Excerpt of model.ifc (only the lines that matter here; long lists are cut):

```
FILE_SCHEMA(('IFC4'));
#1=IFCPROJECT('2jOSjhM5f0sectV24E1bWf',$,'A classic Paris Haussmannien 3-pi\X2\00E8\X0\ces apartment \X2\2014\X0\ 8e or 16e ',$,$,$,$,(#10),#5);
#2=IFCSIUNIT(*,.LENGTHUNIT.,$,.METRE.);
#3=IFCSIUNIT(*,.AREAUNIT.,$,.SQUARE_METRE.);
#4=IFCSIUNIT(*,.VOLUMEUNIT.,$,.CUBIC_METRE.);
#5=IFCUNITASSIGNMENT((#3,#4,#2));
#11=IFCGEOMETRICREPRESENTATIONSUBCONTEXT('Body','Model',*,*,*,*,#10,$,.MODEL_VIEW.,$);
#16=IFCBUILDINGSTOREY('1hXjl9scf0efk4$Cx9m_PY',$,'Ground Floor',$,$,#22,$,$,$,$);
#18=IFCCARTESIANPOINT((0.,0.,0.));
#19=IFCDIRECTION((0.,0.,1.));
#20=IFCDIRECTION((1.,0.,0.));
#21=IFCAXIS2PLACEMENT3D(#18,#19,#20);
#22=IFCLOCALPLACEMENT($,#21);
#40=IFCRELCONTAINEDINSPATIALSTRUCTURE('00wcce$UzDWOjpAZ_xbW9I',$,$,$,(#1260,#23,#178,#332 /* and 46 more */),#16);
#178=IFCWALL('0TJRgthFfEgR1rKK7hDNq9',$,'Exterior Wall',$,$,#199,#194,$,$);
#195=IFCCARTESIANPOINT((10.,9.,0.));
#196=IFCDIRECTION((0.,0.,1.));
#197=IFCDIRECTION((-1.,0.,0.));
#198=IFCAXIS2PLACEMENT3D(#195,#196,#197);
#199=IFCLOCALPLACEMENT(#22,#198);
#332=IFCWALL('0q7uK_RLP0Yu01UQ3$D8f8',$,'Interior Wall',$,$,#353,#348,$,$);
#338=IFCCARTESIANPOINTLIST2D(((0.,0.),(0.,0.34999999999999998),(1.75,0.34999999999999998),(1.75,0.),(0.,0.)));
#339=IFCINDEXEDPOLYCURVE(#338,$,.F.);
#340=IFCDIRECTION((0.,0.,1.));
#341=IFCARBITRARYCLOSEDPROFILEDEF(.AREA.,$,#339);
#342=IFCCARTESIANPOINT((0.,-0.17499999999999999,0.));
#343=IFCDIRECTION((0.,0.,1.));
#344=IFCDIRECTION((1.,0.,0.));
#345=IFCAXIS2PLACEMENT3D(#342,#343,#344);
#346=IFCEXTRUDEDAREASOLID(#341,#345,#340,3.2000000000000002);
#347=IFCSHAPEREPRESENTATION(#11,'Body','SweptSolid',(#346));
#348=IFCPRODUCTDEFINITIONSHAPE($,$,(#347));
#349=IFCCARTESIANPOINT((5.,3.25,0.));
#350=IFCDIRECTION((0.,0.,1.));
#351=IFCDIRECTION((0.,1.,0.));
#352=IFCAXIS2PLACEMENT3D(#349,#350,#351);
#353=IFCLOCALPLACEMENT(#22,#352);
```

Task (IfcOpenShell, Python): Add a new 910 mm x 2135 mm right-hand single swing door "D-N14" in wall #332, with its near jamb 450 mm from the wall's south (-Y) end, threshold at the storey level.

```python
import numpy as np
import ifcopenshell
import ifcopenshell.api.feature
import ifcopenshell.api.geometry
import ifcopenshell.api.root
import ifcopenshell.api.spatial
import ifcopenshell.geom
import ifcopenshell.util.element
import ifcopenshell.util.placement
import ifcopenshell.util.representation
import ifcopenshell.util.shape
import ifcopenshell.util.unit

model = ifcopenshell.open("model.ifc")
unit_scale = ifcopenshell.util.unit.calculate_unit_scale(model)
settings = ifcopenshell.geom.settings()


def volume(element):
    """Net volume in cubic metres, openings subtracted."""
    shape = ifcopenshell.geom.create_shape(settings, element)
    return ifcopenshell.util.shape.get_volume(shape.geometry)


wall = model.by_guid("0q7uK_RLP0Yu01UQ3$D8f8")
storey = ifcopenshell.util.element.get_container(wall, ifc_class="IfcBuildingStorey")
context = ifcopenshell.util.representation.get_context(model, "Model", "Body", "MODEL_VIEW")
before = volume(wall)

width, height, from_end, sill = 0.91, 2.135, 0.45, 0.0  # metres

# The wall runs along its own X axis, and the end named is its -X end.
wall_shape = ifcopenshell.geom.create_shape(settings, wall)
x, y, z = ifcopenshell.util.shape.get_vertices(wall_shape.geometry).T
start = x.min() + from_end
face, thickness = float(y.min()), float(y.max() - y.min())
wall_matrix = ifcopenshell.util.placement.get_local_placement(wall.ObjectPlacement)
level = ifcopenshell.util.placement.get_local_placement(storey.ObjectPlacement)[2, 3]


def in_wall(x, y):
    """Placement at x, y metres in the wall's axes, at sill height."""
    matrix = wall_matrix.copy()
    matrix[:, 3] = wall_matrix @ np.array([x / unit_scale, y / unit_scale, 0.0, 1.0])
    matrix[2, 3] = level + sill / unit_scale
    return matrix


# Opening: a box that overshoots both wall faces by 50 mm.
opening = ifcopenshell.api.root.create_entity(model, ifc_class="IfcOpeningElement", predefined_type="OPENING")
box = ifcopenshell.api.geometry.add_wall_representation(
    model, context=context, length=width, height=height, thickness=thickness + 0.1
)
ifcopenshell.api.geometry.assign_representation(model, product=opening, representation=box)
ifcopenshell.api.geometry.edit_object_placement(model, product=opening, matrix=in_wall(start, face - 0.05), is_si=False)
ifcopenshell.api.feature.add_feature(model, feature=opening, element=wall)

door = ifcopenshell.api.root.create_entity(model, ifc_class="IfcDoor", name="D-N14", predefined_type="DOOR")
door.OverallWidth, door.OverallHeight = width / unit_scale, height / unit_scale
door.OperationType = "SINGLE_SWING_RIGHT"
body = ifcopenshell.api.geometry.add_door_representation(
    model,
    context=context,
    overall_width=door.OverallWidth,
    overall_height=door.OverallHeight,
    operation_type="SINGLE_SWING_RIGHT",
    lining_properties={"LiningDepth": thickness / unit_scale, "ThresholdDepth": thickness / unit_scale},
)
ifcopenshell.api.geometry.assign_representation(model, product=door, representation=body)
ifcopenshell.api.spatial.assign_container(model, products=[door], relating_structure=storey)
ifcopenshell.api.feature.add_filling(model, opening=opening, element=door)

# The lining spans the wall, so the door starts at the wall face.
ifcopenshell.api.geometry.edit_object_placement(model, product=door, matrix=in_wall(start, face), is_si=False)

after = volume(wall)

print(f"wall volume {before:.3f} -> {after:.3f} m3")

model.write("model_edited.ifc")
```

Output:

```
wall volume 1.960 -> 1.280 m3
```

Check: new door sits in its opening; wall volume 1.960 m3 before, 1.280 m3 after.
